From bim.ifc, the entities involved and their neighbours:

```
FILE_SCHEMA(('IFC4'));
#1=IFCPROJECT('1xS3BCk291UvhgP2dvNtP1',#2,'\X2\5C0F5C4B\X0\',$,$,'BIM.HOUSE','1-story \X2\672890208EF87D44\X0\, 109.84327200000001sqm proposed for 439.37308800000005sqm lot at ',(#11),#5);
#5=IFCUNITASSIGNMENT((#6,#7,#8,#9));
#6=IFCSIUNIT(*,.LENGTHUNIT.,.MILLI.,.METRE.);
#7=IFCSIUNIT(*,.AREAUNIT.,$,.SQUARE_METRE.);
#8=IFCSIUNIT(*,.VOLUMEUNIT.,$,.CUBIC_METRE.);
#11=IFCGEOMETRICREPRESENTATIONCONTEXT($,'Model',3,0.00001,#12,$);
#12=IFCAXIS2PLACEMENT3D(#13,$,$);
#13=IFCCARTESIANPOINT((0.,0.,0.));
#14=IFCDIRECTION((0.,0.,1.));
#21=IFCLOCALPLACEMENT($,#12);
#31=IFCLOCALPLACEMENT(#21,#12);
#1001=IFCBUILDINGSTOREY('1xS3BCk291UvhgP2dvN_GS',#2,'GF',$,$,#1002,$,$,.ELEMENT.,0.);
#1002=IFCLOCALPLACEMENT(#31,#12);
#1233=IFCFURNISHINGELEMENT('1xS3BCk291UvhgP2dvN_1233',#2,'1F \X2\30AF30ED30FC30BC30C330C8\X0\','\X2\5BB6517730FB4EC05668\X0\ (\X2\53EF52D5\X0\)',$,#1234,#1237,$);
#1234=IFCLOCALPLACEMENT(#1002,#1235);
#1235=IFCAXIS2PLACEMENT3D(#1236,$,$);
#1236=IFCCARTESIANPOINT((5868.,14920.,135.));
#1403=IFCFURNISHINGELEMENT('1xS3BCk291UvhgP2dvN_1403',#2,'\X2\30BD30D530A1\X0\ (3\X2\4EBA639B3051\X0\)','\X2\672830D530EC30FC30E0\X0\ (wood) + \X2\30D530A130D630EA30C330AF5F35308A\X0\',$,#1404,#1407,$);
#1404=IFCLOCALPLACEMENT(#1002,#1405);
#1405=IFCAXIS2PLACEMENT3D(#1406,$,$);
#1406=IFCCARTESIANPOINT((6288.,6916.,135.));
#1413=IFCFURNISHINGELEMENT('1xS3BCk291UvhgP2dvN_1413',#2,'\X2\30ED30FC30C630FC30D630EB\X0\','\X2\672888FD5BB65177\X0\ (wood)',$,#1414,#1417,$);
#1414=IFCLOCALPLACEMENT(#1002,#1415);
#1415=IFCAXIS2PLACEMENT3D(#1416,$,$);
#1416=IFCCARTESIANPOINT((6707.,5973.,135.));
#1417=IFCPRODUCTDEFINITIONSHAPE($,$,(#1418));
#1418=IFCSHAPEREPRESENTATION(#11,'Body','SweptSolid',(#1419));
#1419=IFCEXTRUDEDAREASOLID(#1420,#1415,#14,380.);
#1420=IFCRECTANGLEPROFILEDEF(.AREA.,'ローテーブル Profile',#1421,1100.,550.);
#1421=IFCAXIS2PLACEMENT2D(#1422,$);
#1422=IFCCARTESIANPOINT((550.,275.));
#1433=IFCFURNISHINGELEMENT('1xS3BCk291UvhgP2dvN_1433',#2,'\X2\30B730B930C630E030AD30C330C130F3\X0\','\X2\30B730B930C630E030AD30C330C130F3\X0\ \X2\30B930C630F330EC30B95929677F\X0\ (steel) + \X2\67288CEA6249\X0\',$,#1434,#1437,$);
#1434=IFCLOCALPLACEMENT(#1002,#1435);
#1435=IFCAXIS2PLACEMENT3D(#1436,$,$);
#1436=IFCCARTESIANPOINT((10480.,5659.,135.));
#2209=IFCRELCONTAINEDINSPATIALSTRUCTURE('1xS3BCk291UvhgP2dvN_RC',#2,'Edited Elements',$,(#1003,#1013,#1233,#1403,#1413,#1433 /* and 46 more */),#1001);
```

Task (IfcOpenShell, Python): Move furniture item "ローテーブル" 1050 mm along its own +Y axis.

```python
import ifcopenshell
import ifcopenshell.api.geometry
import ifcopenshell.util.placement
import ifcopenshell.util.unit

model = ifcopenshell.open("bim.ifc")
unit_scale = ifcopenshell.util.unit.calculate_unit_scale(model)

item = model.by_guid("1xS3BCk291UvhgP2dvN_1413")
matrix = ifcopenshell.util.placement.get_local_placement(item.ObjectPlacement)
matrix[:3, 3] += matrix[:3, 1] * 1.05 / unit_scale
ifcopenshell.api.geometry.edit_object_placement(model, product=item, matrix=matrix, is_si=False)

print(ifcopenshell.util.placement.get_local_placement(item.ObjectPlacement).round(3) + 0.0)

model.write("bim-out.ifc")
```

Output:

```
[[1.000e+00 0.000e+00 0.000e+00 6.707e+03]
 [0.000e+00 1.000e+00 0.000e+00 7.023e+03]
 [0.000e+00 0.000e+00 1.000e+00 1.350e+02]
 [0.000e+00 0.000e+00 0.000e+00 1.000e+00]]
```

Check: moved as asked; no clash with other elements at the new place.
